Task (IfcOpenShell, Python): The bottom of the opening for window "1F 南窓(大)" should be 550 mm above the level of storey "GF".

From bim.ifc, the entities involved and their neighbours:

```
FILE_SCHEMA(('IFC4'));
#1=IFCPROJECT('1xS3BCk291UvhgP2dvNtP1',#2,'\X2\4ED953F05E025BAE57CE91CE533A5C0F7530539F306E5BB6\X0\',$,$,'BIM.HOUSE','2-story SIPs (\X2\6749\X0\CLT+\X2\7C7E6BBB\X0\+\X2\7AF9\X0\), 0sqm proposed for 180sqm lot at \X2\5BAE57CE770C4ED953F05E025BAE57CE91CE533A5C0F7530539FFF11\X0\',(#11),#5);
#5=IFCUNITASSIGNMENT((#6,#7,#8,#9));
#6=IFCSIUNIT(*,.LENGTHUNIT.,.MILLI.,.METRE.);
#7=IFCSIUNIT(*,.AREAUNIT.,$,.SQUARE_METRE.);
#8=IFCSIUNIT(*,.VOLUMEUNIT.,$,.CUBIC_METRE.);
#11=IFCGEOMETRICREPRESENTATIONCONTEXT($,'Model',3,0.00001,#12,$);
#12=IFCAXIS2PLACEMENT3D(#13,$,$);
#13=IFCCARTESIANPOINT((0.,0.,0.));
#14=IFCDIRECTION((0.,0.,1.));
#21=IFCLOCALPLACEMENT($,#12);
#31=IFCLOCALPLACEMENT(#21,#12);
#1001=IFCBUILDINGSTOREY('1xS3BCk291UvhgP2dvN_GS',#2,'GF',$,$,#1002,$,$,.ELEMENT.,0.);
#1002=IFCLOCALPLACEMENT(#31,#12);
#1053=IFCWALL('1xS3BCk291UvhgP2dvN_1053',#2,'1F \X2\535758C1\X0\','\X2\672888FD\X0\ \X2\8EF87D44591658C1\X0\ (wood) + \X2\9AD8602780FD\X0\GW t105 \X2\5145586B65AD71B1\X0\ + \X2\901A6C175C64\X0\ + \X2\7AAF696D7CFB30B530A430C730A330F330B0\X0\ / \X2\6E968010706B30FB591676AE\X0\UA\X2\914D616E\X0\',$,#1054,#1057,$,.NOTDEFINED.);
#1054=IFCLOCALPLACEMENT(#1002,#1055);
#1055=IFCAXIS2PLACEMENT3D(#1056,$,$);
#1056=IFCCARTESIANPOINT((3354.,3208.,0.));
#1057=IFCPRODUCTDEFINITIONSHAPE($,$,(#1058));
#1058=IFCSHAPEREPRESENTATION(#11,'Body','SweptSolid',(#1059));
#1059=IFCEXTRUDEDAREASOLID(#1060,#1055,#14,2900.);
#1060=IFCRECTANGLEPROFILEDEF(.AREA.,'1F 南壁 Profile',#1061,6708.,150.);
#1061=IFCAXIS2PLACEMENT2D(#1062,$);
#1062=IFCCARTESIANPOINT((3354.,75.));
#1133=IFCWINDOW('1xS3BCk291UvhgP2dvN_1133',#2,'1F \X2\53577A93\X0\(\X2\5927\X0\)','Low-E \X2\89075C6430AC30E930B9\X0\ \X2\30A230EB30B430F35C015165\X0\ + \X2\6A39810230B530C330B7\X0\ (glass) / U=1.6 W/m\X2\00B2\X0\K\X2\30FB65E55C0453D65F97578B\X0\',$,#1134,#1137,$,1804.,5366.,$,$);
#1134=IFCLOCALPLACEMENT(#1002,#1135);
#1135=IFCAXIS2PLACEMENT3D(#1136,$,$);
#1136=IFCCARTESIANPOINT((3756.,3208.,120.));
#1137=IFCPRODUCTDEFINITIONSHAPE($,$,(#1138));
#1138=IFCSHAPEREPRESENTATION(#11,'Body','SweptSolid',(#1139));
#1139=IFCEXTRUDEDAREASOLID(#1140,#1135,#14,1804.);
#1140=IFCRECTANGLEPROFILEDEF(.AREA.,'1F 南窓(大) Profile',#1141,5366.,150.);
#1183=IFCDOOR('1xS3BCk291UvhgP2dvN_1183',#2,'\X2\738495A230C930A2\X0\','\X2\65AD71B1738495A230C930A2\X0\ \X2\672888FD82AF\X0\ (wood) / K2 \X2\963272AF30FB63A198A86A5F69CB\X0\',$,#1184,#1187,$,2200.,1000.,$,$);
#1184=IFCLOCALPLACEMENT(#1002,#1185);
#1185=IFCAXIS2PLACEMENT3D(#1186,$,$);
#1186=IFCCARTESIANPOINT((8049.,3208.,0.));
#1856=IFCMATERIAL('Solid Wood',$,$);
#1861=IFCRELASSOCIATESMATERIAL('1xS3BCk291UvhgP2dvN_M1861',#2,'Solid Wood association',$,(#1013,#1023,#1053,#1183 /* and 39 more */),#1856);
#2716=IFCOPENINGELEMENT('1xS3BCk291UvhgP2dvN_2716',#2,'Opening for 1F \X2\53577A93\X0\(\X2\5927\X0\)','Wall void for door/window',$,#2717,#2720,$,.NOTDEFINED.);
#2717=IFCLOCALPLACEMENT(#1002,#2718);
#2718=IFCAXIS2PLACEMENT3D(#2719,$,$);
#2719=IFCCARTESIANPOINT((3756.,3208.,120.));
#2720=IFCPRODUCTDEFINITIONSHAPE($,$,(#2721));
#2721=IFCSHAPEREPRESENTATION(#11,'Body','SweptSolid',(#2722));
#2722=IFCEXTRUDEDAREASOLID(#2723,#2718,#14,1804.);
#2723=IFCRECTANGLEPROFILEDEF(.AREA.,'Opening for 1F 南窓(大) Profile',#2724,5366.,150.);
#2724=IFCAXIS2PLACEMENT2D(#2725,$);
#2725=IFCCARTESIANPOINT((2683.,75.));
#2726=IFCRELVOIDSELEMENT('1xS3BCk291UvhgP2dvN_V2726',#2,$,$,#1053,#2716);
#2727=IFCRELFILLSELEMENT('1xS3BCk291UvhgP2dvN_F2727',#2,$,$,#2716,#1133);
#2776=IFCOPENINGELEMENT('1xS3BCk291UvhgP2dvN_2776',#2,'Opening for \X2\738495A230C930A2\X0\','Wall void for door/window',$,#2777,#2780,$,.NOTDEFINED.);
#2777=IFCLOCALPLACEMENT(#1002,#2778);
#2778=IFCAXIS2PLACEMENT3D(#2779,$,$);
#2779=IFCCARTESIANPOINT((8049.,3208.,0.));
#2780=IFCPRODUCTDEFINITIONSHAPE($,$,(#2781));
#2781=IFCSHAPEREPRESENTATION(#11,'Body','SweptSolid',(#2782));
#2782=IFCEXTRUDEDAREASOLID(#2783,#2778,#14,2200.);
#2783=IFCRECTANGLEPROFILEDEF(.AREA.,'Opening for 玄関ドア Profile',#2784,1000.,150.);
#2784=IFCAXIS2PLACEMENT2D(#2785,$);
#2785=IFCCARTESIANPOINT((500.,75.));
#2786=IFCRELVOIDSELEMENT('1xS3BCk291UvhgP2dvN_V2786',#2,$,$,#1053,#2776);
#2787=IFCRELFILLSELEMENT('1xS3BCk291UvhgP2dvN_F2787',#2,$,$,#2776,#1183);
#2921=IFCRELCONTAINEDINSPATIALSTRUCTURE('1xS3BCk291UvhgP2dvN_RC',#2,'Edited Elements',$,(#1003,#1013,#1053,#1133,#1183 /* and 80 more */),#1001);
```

```python
import numpy as np
import ifcopenshell
import ifcopenshell.api.geometry
import ifcopenshell.geom
import ifcopenshell.util.element
import ifcopenshell.util.placement
import ifcopenshell.util.shape
import ifcopenshell.util.unit

model = ifcopenshell.open("bim.ifc")
unit_scale = ifcopenshell.util.unit.calculate_unit_scale(model)

window = model.by_guid("1xS3BCk291UvhgP2dvN_1133")
opening = window.FillsVoids[0].RelatingOpeningElement
storey = ifcopenshell.util.element.get_container(window, ifc_class="IfcBuildingStorey")
level = ifcopenshell.util.placement.get_local_placement(storey.ObjectPlacement)[2, 3]

# The opening's origin need not be at the sill, so measure its lowest point.
shape = ifcopenshell.geom.create_shape(ifcopenshell.geom.settings(), opening)
bottom = ifcopenshell.util.shape.get_shape_bottom_elevation(shape, shape.geometry) / unit_scale
dz = level + 550.0 - bottom

shift = np.array([0.0, 0.0, dz])
# The window is not placed relative to its opening, so move both.
for product in (opening, window):
    matrix = ifcopenshell.util.placement.get_local_placement(product.ObjectPlacement)
    matrix[:3, 3] += shift
    ifcopenshell.api.geometry.edit_object_placement(model, product=product, matrix=matrix, is_si=False)

print(f"moved by {dz * unit_scale:+.3f} m")

model.write("bim_v2.ifc")
```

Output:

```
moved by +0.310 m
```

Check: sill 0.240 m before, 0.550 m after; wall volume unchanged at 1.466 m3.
